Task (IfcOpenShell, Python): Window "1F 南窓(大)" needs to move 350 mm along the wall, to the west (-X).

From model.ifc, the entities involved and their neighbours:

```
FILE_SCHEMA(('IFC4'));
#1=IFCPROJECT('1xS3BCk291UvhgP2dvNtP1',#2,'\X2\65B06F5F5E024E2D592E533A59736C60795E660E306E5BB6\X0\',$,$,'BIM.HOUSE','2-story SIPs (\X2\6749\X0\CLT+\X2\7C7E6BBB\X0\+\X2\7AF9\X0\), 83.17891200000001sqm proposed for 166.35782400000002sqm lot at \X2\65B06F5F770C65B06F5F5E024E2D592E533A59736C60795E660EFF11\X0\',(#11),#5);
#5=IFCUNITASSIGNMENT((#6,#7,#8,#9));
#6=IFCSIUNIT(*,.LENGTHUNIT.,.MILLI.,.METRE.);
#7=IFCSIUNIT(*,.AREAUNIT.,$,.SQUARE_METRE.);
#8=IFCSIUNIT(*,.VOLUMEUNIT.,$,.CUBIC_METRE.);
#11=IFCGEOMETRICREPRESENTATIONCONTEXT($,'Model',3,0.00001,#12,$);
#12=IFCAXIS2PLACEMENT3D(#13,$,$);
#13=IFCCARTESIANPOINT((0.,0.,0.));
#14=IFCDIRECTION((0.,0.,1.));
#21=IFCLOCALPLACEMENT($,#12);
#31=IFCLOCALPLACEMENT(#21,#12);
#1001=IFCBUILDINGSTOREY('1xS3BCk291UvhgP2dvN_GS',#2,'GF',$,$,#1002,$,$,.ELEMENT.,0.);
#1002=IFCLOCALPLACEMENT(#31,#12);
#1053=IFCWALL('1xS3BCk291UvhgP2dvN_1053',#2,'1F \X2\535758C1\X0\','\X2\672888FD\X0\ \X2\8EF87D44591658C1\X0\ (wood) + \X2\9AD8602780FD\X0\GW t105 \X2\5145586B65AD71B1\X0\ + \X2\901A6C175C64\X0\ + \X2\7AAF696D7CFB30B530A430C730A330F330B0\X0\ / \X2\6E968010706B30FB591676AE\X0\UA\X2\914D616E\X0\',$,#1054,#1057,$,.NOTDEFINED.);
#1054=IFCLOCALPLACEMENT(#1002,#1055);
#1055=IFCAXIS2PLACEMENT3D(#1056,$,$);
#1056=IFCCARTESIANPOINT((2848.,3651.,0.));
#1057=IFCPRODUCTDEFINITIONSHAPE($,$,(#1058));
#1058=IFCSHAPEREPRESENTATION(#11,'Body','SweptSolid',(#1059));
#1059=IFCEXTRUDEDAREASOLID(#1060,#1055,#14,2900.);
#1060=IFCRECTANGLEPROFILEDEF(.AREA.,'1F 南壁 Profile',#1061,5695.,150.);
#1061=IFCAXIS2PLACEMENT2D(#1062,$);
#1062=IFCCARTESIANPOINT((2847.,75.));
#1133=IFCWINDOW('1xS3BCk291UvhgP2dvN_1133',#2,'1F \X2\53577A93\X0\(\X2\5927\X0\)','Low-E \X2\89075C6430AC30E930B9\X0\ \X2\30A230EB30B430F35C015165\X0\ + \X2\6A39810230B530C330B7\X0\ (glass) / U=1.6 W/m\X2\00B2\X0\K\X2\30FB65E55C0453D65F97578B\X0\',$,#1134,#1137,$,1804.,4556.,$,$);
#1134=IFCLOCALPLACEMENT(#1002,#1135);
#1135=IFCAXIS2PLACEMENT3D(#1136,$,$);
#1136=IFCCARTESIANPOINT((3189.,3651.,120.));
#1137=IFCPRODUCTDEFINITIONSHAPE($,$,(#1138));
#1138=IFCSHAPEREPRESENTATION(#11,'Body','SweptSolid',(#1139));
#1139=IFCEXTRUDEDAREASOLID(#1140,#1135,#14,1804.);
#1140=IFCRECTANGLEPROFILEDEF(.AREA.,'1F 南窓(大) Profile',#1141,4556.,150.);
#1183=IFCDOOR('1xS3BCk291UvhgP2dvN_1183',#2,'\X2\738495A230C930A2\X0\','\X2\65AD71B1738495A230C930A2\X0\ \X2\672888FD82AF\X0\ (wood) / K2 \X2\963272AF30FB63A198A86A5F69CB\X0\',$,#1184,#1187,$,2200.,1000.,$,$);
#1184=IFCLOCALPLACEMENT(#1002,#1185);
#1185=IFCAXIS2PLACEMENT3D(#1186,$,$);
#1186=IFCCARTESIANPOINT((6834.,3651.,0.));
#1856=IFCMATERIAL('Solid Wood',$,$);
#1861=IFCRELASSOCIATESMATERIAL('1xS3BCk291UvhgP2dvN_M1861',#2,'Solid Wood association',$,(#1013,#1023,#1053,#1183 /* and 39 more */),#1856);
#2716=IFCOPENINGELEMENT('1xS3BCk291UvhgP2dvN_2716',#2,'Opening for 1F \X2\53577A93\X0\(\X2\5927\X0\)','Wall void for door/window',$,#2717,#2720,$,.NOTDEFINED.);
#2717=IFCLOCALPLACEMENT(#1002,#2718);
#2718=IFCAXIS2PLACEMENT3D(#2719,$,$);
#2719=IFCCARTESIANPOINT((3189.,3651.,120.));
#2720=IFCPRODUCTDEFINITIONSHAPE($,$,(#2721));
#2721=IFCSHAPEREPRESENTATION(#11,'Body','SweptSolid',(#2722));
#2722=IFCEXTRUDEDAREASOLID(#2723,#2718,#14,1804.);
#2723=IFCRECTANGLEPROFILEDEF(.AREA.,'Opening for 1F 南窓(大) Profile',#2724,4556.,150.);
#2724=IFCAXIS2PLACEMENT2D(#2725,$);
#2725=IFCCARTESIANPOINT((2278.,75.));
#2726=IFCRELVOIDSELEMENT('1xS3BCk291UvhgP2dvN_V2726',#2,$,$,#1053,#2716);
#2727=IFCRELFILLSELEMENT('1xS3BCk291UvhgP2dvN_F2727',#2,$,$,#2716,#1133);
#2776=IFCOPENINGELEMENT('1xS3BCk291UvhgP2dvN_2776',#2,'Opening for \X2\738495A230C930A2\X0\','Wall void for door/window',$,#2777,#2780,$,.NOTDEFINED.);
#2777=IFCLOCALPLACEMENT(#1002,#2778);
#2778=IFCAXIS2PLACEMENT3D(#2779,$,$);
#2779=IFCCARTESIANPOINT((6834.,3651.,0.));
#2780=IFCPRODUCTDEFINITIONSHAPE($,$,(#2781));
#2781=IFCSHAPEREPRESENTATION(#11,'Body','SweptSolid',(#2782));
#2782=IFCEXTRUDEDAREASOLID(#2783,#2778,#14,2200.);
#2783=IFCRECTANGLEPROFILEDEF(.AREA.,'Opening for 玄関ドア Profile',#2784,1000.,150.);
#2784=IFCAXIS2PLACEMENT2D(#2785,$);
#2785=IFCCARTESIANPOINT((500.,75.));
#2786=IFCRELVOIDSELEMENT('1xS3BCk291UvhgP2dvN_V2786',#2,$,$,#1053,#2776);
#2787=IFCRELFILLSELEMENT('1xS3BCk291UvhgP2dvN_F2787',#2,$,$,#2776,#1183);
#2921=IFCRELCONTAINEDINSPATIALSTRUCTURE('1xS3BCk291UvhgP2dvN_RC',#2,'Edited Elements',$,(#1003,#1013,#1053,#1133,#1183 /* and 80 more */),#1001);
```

```python
import ifcopenshell
import ifcopenshell.api.geometry
import ifcopenshell.util.placement

model = ifcopenshell.open("model.ifc")

window = model.by_guid("1xS3BCk291UvhgP2dvN_1133")
opening = window.FillsVoids[0].RelatingOpeningElement
wall = opening.VoidsElements[0].RelatingBuildingElement

wall_matrix = ifcopenshell.util.placement.get_local_placement(wall.ObjectPlacement)
shift = wall_matrix[:3, 0] * -350.0
before = ifcopenshell.util.placement.get_local_placement(window.ObjectPlacement)[:3, 3].copy()

# The window is not placed relative to its opening, so move both.
for product in (opening, window):
    matrix = ifcopenshell.util.placement.get_local_placement(product.ObjectPlacement)
    matrix[:3, 3] += shift
    ifcopenshell.api.geometry.edit_object_placement(model, product=product, matrix=matrix, is_si=False)

after = ifcopenshell.util.placement.get_local_placement(window.ObjectPlacement)[:3, 3]
print("window moved by", (after - before).round(3) + 0.0)

model.write("model_rev.ifc")
```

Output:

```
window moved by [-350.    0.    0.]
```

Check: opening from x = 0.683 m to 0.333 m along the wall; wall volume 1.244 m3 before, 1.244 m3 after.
